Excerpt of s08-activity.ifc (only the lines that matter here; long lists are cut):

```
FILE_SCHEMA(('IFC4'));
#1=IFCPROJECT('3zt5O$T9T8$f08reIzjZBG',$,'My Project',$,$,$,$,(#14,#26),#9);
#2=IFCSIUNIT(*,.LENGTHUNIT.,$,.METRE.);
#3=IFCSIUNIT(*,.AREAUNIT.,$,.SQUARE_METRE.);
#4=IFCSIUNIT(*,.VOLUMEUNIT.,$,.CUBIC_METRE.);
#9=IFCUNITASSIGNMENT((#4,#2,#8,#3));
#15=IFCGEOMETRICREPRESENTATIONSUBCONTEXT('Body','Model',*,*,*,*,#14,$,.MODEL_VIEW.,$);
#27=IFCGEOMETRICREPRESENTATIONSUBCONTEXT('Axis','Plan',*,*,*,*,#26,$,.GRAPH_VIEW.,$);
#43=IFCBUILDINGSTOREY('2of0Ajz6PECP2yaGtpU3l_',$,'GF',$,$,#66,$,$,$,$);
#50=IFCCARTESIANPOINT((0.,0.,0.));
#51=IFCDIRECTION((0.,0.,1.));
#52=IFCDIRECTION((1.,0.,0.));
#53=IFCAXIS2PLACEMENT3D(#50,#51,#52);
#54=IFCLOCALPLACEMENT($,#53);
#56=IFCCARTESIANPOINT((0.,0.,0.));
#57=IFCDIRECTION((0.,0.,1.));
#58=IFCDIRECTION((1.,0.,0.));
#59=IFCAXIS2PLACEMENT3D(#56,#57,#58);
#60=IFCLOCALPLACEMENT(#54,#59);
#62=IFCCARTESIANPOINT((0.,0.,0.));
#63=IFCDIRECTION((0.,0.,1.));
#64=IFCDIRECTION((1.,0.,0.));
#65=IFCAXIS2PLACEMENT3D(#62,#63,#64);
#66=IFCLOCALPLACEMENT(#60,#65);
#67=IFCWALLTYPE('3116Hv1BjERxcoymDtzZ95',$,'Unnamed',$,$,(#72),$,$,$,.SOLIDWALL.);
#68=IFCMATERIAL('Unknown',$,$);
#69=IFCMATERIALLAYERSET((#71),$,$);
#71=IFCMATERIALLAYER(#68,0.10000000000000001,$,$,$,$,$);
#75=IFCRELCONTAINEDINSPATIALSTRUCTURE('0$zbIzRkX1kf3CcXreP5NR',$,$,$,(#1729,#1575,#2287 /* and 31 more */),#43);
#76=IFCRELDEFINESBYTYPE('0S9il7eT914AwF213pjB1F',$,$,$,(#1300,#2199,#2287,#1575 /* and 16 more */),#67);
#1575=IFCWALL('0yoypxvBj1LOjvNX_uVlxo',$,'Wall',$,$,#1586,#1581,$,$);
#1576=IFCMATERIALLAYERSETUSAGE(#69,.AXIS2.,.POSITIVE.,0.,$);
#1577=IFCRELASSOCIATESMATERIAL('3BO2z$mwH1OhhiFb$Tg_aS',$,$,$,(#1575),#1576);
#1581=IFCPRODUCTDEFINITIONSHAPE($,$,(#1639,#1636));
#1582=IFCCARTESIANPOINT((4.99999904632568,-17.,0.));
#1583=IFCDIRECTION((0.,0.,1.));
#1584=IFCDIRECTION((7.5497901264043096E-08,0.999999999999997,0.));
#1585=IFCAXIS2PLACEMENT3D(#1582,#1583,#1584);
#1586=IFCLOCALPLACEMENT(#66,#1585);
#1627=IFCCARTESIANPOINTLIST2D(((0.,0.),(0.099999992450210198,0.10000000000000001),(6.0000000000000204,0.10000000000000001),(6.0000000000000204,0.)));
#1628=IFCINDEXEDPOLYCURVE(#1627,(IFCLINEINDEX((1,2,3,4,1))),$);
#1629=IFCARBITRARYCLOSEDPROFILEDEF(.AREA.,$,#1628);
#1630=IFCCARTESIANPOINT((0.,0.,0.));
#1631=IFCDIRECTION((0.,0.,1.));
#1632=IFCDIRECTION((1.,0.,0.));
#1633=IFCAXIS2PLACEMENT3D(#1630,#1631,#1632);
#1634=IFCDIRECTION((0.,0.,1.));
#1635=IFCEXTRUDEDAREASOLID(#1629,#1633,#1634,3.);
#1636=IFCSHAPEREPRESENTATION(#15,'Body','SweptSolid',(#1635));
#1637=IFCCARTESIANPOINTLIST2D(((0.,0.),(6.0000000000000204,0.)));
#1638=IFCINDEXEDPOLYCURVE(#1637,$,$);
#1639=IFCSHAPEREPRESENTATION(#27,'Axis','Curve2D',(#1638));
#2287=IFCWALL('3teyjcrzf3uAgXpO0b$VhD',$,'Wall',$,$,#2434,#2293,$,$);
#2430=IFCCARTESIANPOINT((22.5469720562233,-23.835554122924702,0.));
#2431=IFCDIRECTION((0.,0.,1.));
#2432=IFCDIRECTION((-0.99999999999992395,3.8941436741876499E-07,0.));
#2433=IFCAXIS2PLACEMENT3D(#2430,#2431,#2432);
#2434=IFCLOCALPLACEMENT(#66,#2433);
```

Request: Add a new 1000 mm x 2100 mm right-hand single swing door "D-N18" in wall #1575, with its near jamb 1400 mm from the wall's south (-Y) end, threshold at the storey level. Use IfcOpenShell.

```python
import numpy as np
import ifcopenshell
import ifcopenshell.api.feature
import ifcopenshell.api.geometry
import ifcopenshell.api.root
import ifcopenshell.api.spatial
import ifcopenshell.geom
import ifcopenshell.util.element
import ifcopenshell.util.placement
import ifcopenshell.util.representation
import ifcopenshell.util.shape
import ifcopenshell.util.unit

model = ifcopenshell.open("s08-activity.ifc")
unit_scale = ifcopenshell.util.unit.calculate_unit_scale(model)
settings = ifcopenshell.geom.settings()


def volume(element):
    """Net volume in cubic metres, openings subtracted."""
    shape = ifcopenshell.geom.create_shape(settings, element)
    return ifcopenshell.util.shape.get_volume(shape.geometry)


wall = model.by_guid("0yoypxvBj1LOjvNX_uVlxo")
storey = ifcopenshell.util.element.get_container(wall, ifc_class="IfcBuildingStorey")
context = ifcopenshell.util.representation.get_context(model, "Model", "Body", "MODEL_VIEW")
before = volume(wall)

width, height, from_end, sill = 1, 2.1, 1.4, 0.0  # metres

# The wall runs along its own X axis, and the end named is its -X end.
wall_shape = ifcopenshell.geom.create_shape(settings, wall)
x, y, z = ifcopenshell.util.shape.get_vertices(wall_shape.geometry).T
start = x.min() + from_end
face, thickness = float(y.min()), float(y.max() - y.min())
wall_matrix = ifcopenshell.util.placement.get_local_placement(wall.ObjectPlacement)
level = ifcopenshell.util.placement.get_local_placement(storey.ObjectPlacement)[2, 3]


def in_wall(x, y):
    """Placement at x, y metres in the wall's axes, at sill height."""
    matrix = wall_matrix.copy()
    matrix[:, 3] = wall_matrix @ np.array([x / unit_scale, y / unit_scale, 0.0, 1.0])
    matrix[2, 3] = level + sill / unit_scale
    return matrix


# Opening: a box that overshoots both wall faces by 50 mm.
opening = ifcopenshell.api.root.create_entity(model, ifc_class="IfcOpeningElement", predefined_type="OPENING")
box = ifcopenshell.api.geometry.add_wall_representation(
    model, context=context, length=width, height=height, thickness=thickness + 0.1
)
ifcopenshell.api.geometry.assign_representation(model, product=opening, representation=box)
ifcopenshell.api.geometry.edit_object_placement(model, product=opening, matrix=in_wall(start, face - 0.05), is_si=False)
ifcopenshell.api.feature.add_feature(model, feature=opening, element=wall)

door = ifcopenshell.api.root.create_entity(model, ifc_class="IfcDoor", name="D-N18", predefined_type="DOOR")
door.OverallWidth, door.OverallHeight = width / unit_scale, height / unit_scale
door.OperationType = "SINGLE_SWING_RIGHT"
body = ifcopenshell.api.geometry.add_door_representation(
    model,
    context=context,
    overall_width=door.OverallWidth,
    overall_height=door.OverallHeight,
    operation_type="SINGLE_SWING_RIGHT",
    lining_properties={"LiningDepth": thickness / unit_scale, "ThresholdDepth": thickness / unit_scale},
)
ifcopenshell.api.geometry.assign_representation(model, product=door, representation=body)
ifcopenshell.api.spatial.assign_container(model, products=[door], relating_structure=storey)
ifcopenshell.api.feature.add_filling(model, opening=opening, element=door)

# The lining spans the wall, so the door starts at the wall face.
ifcopenshell.api.geometry.edit_object_placement(model, product=door, matrix=in_wall(start, face), is_si=False)

after = volume(wall)

print(f"wall volume {before:.3f} -> {after:.3f} m3")

model.write("s08-activity_edited.ifc")
```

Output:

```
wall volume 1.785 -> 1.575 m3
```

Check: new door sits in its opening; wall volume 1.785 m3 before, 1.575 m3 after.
